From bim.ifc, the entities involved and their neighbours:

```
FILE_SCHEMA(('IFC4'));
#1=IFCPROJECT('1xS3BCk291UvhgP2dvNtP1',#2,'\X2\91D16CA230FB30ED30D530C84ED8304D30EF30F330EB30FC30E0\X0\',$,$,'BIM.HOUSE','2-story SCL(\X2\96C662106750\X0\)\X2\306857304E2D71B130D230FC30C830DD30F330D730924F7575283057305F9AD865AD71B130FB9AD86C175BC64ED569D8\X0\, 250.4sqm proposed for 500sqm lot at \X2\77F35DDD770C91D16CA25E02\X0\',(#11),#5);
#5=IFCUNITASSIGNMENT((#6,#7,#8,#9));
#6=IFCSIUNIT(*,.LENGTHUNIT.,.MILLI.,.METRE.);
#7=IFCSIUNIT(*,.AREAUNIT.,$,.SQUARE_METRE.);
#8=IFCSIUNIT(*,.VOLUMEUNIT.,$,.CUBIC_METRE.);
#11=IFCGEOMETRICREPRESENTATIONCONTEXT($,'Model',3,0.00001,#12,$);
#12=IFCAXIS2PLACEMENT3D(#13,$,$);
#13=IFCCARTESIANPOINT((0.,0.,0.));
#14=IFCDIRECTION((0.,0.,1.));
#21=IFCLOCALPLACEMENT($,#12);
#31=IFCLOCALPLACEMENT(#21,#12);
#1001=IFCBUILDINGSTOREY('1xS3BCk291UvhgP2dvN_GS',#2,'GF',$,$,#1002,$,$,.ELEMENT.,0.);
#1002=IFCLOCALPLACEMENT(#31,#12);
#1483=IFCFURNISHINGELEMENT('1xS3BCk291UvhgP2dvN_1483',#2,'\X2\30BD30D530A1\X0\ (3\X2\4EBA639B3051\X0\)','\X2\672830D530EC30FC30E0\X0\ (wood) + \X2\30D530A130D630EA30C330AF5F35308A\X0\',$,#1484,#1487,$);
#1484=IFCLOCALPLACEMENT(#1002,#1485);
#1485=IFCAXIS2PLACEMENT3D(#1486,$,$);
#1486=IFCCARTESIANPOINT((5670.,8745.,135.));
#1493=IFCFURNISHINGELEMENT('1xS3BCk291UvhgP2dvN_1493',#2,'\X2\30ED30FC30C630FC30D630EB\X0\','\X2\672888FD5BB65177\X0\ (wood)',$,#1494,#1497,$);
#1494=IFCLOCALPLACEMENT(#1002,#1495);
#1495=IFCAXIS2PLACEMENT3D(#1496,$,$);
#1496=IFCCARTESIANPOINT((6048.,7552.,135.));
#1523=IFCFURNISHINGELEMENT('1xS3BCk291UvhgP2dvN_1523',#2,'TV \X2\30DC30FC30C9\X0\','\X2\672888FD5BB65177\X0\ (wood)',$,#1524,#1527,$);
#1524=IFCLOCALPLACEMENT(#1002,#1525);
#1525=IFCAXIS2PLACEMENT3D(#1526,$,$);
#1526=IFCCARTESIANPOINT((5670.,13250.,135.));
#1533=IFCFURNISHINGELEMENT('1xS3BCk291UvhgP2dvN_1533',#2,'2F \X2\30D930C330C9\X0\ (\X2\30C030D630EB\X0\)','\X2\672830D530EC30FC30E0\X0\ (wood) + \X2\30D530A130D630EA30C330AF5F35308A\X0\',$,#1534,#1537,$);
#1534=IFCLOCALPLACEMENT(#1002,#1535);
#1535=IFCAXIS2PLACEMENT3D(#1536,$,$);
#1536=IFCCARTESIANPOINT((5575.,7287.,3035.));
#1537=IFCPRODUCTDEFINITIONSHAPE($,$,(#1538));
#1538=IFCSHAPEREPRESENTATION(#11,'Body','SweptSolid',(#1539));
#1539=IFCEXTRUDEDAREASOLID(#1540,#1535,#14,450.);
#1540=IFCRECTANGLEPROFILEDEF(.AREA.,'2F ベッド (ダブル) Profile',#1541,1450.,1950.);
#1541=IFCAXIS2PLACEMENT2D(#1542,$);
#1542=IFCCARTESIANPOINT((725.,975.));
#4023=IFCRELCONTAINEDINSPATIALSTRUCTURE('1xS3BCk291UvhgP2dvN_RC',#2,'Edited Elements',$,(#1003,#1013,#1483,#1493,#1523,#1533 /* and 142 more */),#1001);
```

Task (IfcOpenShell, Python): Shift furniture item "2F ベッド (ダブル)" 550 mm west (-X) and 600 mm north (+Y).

```python
import ifcopenshell
import ifcopenshell.api.geometry
import ifcopenshell.util.placement
import ifcopenshell.util.unit

model = ifcopenshell.open("bim.ifc")
unit_scale = ifcopenshell.util.unit.calculate_unit_scale(model)

item = model.by_id(1533)
matrix = ifcopenshell.util.placement.get_local_placement(item.ObjectPlacement)
matrix[0, 3] -= 0.55 / unit_scale
matrix[1, 3] += 0.6 / unit_scale
ifcopenshell.api.geometry.edit_object_placement(model, product=item, matrix=matrix, is_si=False)

print(ifcopenshell.util.placement.get_local_placement(item.ObjectPlacement).round(3) + 0.0)

model.write("bim_updated.ifc")
```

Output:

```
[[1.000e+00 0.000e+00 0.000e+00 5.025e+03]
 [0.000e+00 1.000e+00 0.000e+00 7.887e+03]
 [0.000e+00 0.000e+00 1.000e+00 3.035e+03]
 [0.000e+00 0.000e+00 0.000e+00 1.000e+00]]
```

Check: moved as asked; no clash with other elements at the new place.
